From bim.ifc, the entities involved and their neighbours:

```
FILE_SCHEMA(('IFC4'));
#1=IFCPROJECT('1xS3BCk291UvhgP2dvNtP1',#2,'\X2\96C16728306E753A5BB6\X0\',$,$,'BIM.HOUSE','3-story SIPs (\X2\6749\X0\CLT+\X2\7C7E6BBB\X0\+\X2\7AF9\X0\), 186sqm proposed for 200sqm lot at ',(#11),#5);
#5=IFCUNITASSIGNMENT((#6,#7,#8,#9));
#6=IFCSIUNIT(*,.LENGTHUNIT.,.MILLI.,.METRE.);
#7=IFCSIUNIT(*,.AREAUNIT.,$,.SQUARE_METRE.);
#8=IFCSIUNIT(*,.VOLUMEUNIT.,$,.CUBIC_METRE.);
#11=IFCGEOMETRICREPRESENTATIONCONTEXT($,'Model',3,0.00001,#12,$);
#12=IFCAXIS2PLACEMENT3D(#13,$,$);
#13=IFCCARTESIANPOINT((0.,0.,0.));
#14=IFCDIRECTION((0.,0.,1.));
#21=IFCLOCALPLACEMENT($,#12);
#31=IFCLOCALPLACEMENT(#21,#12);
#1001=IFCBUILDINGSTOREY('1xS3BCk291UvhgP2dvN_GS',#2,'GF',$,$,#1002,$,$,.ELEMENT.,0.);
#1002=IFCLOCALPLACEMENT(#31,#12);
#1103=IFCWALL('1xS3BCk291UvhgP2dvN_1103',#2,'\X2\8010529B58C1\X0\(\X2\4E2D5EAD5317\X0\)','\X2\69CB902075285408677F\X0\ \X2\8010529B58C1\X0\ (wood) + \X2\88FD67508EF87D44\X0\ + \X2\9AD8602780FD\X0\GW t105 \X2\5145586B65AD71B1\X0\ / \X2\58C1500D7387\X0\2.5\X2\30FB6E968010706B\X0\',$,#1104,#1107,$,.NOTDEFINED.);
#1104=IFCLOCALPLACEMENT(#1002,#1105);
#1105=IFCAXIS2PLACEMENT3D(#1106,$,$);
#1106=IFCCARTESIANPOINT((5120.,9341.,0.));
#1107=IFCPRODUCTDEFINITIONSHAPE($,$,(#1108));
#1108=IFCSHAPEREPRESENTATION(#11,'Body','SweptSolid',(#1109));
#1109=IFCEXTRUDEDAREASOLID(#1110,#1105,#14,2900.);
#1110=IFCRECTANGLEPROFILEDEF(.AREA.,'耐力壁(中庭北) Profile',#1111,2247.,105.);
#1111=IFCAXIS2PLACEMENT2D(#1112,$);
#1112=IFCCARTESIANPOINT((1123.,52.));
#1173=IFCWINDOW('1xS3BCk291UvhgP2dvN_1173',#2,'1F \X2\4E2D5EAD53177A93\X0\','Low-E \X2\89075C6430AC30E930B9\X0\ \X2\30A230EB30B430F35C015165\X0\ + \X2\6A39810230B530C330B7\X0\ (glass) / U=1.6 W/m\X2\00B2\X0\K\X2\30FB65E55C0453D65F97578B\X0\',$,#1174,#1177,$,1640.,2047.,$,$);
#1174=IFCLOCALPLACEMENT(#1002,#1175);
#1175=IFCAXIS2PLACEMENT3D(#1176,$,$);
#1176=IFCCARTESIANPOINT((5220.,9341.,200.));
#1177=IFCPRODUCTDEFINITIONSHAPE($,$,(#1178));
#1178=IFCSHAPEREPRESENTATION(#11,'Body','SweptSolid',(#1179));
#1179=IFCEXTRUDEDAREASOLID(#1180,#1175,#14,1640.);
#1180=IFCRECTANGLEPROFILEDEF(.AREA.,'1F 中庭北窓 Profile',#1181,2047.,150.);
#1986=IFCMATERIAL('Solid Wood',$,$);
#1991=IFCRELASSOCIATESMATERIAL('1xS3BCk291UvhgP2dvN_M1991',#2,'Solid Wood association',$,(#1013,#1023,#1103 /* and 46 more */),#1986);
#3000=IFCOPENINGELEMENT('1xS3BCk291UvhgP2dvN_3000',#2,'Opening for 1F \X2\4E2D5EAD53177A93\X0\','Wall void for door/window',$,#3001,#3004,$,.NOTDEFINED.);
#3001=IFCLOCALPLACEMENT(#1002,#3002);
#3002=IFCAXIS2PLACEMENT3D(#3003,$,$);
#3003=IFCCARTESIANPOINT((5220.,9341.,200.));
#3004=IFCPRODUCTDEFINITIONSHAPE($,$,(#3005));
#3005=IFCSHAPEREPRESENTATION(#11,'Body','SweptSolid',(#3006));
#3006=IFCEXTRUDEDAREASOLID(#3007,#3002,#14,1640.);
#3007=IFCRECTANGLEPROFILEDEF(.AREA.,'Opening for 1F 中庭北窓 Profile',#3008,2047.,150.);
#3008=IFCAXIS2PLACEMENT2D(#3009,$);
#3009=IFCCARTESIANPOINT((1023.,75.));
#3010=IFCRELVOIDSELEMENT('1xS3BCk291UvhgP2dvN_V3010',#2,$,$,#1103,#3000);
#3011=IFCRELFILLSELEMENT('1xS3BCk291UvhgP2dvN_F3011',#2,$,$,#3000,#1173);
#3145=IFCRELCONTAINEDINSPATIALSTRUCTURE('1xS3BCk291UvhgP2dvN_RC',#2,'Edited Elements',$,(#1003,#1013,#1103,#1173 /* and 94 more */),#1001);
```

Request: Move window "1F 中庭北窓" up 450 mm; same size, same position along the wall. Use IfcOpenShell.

```python
import numpy as np
import ifcopenshell
import ifcopenshell.api.geometry
import ifcopenshell.util.placement
import ifcopenshell.util.unit

model = ifcopenshell.open("bim.ifc")
unit_scale = ifcopenshell.util.unit.calculate_unit_scale(model)

window = model.by_guid("1xS3BCk291UvhgP2dvN_1173")
opening = window.FillsVoids[0].RelatingOpeningElement
dz = 0.45 / unit_scale

shift = np.array([0.0, 0.0, dz])
# The window is not placed relative to its opening, so move both.
for product in (opening, window):
    matrix = ifcopenshell.util.placement.get_local_placement(product.ObjectPlacement)
    matrix[:3, 3] += shift
    ifcopenshell.api.geometry.edit_object_placement(model, product=product, matrix=matrix, is_si=False)

print(f"moved by {dz * unit_scale:+.3f} m")

model.write("bim_updated.ifc")
```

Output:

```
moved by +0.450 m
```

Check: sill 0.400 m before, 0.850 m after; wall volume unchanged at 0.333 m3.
